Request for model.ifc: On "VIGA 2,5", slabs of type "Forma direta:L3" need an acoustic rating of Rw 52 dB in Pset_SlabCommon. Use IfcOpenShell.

First a look at what the model holds.

```python
import ifcopenshell
import ifcopenshell.util.element

model = ifcopenshell.open("model.ifc")
print(model.schema)
storey = next(s for s in model.by_type("IfcBuildingStorey") if s.Name == "VIGA 2,5")
slabs = [e for e in ifcopenshell.util.element.get_decomposition(storey) if e.is_a("IfcSlab")]
seen = {}
for e in slabs:
    element_type = ifcopenshell.util.element.get_type(e)
    key = (element_type.Name if element_type != e and element_type else None, ifcopenshell.util.element.get_pset(e, "Pset_SlabCommon", "AcousticRating"))
    seen[key] = seen.get(key, 0) + 1
for (name, value), count in sorted(seen.items(), key=str):
    print(count, "x", name, "|", value)
```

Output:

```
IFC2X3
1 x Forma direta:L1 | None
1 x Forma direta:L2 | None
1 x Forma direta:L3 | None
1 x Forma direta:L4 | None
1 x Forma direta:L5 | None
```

```python
import ifcopenshell
import ifcopenshell.api.pset
import ifcopenshell.util.element

model = ifcopenshell.open("model.ifc")

storey = next(s for s in model.by_type("IfcBuildingStorey") if s.Name == "VIGA 2,5")
slabs = [e for e in ifcopenshell.util.element.get_decomposition(storey) if e.is_a("IfcSlab")]

count = 0
for e in slabs:
    element_type = ifcopenshell.util.element.get_type(e)
    if element_type in (None, e) or element_type.Name != "Forma direta:L3":
        continue
    # add_pset returns the element's existing set when there is one.
    pset = ifcopenshell.api.pset.add_pset(model, product=e, name="Pset_SlabCommon")
    ifcopenshell.api.pset.edit_pset(model, pset=pset, properties={"AcousticRating": "Rw 52 dB"})
    count += 1

print(count, "slabs updated")

model.write("model_edited.ifc")
```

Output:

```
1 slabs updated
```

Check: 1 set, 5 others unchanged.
